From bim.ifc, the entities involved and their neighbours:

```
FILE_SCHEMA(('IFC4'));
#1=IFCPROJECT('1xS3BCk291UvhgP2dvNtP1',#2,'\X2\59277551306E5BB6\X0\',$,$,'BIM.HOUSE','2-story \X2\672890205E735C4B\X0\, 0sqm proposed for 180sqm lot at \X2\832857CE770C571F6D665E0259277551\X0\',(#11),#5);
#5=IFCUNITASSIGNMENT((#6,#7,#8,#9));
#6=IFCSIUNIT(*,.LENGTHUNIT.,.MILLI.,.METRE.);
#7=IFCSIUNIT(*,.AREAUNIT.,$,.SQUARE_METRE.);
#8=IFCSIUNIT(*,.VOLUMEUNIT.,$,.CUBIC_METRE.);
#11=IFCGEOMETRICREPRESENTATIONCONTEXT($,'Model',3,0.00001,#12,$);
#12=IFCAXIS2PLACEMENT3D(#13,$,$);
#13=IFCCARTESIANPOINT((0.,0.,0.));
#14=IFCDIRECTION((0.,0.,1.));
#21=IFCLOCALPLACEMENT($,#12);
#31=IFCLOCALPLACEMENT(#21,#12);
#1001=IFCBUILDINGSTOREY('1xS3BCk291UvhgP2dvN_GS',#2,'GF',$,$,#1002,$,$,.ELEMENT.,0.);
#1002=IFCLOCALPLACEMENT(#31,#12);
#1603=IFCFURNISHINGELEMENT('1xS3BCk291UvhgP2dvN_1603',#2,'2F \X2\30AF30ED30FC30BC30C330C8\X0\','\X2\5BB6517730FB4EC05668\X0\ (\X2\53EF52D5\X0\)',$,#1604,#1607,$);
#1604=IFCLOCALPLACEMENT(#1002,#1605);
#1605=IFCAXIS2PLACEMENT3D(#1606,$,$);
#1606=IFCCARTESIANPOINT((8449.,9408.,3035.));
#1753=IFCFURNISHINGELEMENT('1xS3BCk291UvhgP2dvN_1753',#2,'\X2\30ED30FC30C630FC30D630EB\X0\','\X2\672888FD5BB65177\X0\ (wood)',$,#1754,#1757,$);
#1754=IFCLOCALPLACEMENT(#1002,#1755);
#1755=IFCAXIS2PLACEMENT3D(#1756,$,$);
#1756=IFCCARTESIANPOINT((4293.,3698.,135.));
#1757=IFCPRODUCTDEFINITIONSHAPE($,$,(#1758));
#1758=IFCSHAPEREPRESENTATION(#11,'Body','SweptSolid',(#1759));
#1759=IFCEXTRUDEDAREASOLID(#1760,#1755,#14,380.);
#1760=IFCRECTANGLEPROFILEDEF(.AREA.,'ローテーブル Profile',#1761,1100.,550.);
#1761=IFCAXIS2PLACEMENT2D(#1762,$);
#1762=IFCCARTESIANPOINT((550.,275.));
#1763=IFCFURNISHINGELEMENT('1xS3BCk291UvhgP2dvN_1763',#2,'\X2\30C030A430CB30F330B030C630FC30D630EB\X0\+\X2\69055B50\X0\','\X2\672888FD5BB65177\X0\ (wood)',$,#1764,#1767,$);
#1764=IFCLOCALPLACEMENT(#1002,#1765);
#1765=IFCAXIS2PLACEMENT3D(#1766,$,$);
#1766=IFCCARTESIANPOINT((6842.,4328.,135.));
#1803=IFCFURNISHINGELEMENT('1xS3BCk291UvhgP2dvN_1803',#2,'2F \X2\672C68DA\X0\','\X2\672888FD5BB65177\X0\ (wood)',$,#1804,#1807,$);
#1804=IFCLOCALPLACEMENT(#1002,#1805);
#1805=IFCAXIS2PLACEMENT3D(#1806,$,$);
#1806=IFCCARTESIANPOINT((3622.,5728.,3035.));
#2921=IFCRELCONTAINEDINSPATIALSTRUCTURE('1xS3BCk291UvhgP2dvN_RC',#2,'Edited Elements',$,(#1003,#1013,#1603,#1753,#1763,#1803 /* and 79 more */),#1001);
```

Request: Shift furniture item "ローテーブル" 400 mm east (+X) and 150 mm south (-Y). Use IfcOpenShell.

```python
import ifcopenshell
import ifcopenshell.api.geometry
import ifcopenshell.util.placement
import ifcopenshell.util.unit

model = ifcopenshell.open("bim.ifc")
unit_scale = ifcopenshell.util.unit.calculate_unit_scale(model)

item = model.by_id(1753)
matrix = ifcopenshell.util.placement.get_local_placement(item.ObjectPlacement)
matrix[0, 3] += 0.4 / unit_scale
matrix[1, 3] -= 0.15 / unit_scale
ifcopenshell.api.geometry.edit_object_placement(model, product=item, matrix=matrix, is_si=False)

print(ifcopenshell.util.placement.get_local_placement(item.ObjectPlacement).round(3) + 0.0)

model.write("bim_edited.ifc")
```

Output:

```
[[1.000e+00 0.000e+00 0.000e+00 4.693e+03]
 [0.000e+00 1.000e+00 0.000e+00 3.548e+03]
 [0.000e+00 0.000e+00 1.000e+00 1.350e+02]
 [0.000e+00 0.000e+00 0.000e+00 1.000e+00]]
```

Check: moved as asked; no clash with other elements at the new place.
